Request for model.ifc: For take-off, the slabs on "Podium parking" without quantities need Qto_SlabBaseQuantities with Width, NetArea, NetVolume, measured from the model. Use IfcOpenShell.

First a look at what the model holds.

```python
import ifcopenshell
import ifcopenshell.util.element
import ifcopenshell.util.unit

model = ifcopenshell.open("model.ifc")
print(model.schema)
for unit_type in ("LENGTHUNIT", "AREAUNIT", "VOLUMEUNIT"):
    print(unit_type, ifcopenshell.util.unit.calculate_unit_scale(model, unit_type))
storey = next(s for s in model.by_type("IfcBuildingStorey") if s.Name == "Podium parking")
slabs = [e for e in ifcopenshell.util.element.get_decomposition(storey) if e.is_a("IfcSlab")]
for e in sorted(slabs, key=lambda e: e.id()):
    print(e.id(), e.is_a(), e.Name, list(ifcopenshell.util.element.get_psets(e, qtos_only=True)), sep=" | ")
```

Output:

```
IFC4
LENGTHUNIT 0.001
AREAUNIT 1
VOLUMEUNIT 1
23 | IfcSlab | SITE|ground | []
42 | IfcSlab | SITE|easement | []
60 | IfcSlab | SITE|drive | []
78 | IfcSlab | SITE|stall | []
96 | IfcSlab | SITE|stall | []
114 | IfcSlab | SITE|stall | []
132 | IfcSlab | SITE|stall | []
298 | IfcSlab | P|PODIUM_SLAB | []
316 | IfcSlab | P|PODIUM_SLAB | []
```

```python
import ifcopenshell
import ifcopenshell.api.pset
import ifcopenshell.geom
import ifcopenshell.util.element
import ifcopenshell.util.shape
import ifcopenshell.util.unit

model = ifcopenshell.open("model.ifc")
unit_scale = ifcopenshell.util.unit.calculate_unit_scale(model)
area_scale = ifcopenshell.util.unit.calculate_unit_scale(model, "AREAUNIT")
volume_scale = ifcopenshell.util.unit.calculate_unit_scale(model, "VOLUMEUNIT")
settings = ifcopenshell.geom.settings()

storey = next(s for s in model.by_type("IfcBuildingStorey") if s.Name == "Podium parking")
slabs = [e for e in ifcopenshell.util.element.get_decomposition(storey) if e.is_a("IfcSlab")]

for e in sorted(slabs, key=lambda e: e.id()):
    if ifcopenshell.util.element.get_psets(e, qtos_only=True, should_inherit=False):
        continue
    # Geometry comes back in metres, in the element's own axes.
    shape = ifcopenshell.geom.create_shape(settings, e)
    values = {
        "Width": ifcopenshell.util.shape.get_z(shape.geometry) / unit_scale,
        "NetArea": ifcopenshell.util.shape.get_footprint_area(shape.geometry) / area_scale,
        "NetVolume": ifcopenshell.util.shape.get_volume(shape.geometry) / volume_scale,
    }
    qto = ifcopenshell.api.pset.add_qto(model, product=e, name="Qto_SlabBaseQuantities")
    ifcopenshell.api.pset.edit_qto(model, qto=qto, properties=values)
    print(e.id(), {k: round(v, 3) for k, v in values.items()})

model.write("model_v2.ifc")
```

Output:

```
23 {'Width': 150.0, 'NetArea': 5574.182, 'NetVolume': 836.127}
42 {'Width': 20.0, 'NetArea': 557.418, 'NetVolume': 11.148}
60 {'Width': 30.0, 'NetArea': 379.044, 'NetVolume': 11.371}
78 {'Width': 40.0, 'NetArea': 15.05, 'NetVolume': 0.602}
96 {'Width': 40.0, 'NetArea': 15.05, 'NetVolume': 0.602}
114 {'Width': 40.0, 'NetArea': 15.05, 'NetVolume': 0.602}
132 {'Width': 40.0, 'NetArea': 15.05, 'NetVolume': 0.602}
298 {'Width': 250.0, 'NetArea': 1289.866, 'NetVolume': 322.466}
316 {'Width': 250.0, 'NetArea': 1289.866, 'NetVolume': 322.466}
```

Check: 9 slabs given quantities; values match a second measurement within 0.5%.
